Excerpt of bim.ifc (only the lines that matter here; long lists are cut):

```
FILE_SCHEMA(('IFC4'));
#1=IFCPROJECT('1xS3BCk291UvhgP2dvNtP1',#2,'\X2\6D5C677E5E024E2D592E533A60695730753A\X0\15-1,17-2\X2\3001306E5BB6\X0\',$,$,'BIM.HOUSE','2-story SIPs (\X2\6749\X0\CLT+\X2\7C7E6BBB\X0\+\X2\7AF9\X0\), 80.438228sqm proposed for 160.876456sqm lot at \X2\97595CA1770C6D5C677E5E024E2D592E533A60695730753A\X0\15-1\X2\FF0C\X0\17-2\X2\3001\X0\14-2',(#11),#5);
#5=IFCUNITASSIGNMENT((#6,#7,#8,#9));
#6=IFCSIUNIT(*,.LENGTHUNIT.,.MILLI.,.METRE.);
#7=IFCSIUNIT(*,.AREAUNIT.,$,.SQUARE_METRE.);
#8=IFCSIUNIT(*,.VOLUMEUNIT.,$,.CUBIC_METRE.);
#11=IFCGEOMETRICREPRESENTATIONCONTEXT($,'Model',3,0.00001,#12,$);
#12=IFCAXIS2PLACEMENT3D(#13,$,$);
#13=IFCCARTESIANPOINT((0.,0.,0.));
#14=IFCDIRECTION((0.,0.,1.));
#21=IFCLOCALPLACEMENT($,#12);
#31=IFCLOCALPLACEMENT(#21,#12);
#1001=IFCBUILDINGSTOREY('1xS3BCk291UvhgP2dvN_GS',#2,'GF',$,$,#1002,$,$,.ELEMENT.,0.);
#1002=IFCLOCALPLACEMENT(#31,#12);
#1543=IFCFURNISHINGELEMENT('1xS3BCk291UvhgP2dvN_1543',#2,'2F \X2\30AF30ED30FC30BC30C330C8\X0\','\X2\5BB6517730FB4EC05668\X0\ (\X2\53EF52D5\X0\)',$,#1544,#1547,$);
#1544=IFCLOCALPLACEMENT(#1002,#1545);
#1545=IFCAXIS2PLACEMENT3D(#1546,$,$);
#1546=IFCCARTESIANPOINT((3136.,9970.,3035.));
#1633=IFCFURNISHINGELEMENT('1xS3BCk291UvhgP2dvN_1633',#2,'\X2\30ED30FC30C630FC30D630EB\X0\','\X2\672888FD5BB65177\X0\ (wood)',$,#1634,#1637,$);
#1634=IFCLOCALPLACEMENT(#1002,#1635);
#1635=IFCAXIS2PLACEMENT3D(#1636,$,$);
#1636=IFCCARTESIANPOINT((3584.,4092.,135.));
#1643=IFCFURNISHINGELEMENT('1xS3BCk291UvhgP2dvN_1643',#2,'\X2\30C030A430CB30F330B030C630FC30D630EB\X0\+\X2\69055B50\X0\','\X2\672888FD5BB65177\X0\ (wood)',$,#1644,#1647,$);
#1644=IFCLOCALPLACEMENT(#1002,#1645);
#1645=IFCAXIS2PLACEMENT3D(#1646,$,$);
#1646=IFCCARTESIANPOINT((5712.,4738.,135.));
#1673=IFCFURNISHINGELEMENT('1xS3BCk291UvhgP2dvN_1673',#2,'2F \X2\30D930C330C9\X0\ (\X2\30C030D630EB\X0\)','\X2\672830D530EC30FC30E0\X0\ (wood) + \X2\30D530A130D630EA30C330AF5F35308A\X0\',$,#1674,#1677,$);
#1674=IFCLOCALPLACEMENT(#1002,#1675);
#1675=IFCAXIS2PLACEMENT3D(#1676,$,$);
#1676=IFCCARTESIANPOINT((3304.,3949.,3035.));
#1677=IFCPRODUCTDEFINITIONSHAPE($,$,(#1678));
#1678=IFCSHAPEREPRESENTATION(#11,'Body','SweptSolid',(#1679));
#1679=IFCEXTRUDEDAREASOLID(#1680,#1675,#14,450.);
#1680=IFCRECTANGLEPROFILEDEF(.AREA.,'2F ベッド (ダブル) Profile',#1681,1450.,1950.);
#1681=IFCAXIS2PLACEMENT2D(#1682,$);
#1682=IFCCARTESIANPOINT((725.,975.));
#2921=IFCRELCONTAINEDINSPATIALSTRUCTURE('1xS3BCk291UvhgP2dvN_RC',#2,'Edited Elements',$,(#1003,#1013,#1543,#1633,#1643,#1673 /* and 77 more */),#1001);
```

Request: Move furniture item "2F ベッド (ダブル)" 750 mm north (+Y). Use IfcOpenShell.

```python
import ifcopenshell
import ifcopenshell.api.geometry
import ifcopenshell.util.placement
import ifcopenshell.util.unit

model = ifcopenshell.open("bim.ifc")
unit_scale = ifcopenshell.util.unit.calculate_unit_scale(model)

item = model.by_id(1673)
matrix = ifcopenshell.util.placement.get_local_placement(item.ObjectPlacement)
matrix[1, 3] += 0.75 / unit_scale
ifcopenshell.api.geometry.edit_object_placement(model, product=item, matrix=matrix, is_si=False)

print(ifcopenshell.util.placement.get_local_placement(item.ObjectPlacement).round(3) + 0.0)

model.write("bim_v2.ifc")
```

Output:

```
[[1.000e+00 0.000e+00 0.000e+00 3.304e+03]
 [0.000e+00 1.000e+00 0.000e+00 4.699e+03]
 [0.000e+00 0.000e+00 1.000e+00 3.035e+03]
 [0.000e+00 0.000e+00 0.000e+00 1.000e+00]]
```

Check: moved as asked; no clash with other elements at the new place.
